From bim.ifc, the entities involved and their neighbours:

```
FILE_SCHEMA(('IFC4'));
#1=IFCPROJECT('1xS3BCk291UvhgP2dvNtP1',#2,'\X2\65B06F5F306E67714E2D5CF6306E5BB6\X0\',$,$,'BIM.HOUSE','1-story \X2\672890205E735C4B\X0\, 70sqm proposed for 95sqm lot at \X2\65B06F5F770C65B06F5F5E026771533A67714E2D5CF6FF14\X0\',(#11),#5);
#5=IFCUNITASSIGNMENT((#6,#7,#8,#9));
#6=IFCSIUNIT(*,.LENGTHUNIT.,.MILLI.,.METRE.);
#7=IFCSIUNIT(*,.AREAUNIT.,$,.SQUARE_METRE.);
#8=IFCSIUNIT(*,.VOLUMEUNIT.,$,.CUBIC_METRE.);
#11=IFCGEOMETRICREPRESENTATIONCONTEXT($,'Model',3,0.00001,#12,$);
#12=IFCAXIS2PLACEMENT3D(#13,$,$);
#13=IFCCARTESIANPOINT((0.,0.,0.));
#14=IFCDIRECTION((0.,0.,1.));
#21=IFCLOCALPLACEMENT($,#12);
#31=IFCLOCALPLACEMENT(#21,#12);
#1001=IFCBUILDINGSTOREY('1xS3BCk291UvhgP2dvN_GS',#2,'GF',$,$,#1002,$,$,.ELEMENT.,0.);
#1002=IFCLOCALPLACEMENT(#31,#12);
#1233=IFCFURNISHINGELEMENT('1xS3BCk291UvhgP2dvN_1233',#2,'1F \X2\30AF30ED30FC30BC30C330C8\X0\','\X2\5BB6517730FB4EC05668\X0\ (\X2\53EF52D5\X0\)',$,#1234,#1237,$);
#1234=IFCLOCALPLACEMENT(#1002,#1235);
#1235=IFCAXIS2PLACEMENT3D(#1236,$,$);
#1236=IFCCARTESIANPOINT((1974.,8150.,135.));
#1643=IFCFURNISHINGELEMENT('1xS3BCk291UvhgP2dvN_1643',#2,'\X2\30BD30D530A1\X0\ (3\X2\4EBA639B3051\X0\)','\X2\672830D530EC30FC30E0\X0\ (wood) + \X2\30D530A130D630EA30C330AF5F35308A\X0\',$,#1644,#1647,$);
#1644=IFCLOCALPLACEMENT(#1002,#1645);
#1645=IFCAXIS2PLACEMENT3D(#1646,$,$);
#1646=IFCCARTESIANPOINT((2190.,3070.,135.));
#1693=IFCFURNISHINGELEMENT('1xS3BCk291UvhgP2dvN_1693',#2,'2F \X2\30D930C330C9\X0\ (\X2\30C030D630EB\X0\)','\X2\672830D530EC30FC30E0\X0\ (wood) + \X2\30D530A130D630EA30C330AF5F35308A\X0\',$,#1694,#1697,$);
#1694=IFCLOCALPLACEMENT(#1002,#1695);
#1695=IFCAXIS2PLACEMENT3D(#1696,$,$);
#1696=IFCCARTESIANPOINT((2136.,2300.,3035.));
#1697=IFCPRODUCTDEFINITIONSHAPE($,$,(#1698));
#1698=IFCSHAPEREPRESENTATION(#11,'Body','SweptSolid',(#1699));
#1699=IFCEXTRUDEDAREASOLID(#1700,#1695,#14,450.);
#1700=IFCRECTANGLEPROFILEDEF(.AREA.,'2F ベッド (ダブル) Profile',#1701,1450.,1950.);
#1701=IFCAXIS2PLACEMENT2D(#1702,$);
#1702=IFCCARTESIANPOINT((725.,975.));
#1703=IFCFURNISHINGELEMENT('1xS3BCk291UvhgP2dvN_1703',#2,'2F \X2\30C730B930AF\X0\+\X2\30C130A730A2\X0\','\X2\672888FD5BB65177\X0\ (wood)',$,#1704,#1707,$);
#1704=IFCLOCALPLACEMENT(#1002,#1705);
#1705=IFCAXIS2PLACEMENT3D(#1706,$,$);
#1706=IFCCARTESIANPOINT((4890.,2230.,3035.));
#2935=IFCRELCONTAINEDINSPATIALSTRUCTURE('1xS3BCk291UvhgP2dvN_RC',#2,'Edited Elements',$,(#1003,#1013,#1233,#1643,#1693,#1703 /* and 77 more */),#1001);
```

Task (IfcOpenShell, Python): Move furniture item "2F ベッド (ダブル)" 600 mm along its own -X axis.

```python
import ifcopenshell
import ifcopenshell.api.geometry
import ifcopenshell.util.placement
import ifcopenshell.util.unit

model = ifcopenshell.open("bim.ifc")
unit_scale = ifcopenshell.util.unit.calculate_unit_scale(model)

item = model.by_id(1693)
matrix = ifcopenshell.util.placement.get_local_placement(item.ObjectPlacement)
matrix[:3, 3] -= matrix[:3, 0] * 0.6 / unit_scale
ifcopenshell.api.geometry.edit_object_placement(model, product=item, matrix=matrix, is_si=False)

print(ifcopenshell.util.placement.get_local_placement(item.ObjectPlacement).round(3) + 0.0)

model.write("bim_updated.ifc")
```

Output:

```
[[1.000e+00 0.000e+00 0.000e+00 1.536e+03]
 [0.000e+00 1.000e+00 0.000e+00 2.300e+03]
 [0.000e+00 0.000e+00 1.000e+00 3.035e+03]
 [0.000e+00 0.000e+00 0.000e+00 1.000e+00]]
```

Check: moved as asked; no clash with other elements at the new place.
